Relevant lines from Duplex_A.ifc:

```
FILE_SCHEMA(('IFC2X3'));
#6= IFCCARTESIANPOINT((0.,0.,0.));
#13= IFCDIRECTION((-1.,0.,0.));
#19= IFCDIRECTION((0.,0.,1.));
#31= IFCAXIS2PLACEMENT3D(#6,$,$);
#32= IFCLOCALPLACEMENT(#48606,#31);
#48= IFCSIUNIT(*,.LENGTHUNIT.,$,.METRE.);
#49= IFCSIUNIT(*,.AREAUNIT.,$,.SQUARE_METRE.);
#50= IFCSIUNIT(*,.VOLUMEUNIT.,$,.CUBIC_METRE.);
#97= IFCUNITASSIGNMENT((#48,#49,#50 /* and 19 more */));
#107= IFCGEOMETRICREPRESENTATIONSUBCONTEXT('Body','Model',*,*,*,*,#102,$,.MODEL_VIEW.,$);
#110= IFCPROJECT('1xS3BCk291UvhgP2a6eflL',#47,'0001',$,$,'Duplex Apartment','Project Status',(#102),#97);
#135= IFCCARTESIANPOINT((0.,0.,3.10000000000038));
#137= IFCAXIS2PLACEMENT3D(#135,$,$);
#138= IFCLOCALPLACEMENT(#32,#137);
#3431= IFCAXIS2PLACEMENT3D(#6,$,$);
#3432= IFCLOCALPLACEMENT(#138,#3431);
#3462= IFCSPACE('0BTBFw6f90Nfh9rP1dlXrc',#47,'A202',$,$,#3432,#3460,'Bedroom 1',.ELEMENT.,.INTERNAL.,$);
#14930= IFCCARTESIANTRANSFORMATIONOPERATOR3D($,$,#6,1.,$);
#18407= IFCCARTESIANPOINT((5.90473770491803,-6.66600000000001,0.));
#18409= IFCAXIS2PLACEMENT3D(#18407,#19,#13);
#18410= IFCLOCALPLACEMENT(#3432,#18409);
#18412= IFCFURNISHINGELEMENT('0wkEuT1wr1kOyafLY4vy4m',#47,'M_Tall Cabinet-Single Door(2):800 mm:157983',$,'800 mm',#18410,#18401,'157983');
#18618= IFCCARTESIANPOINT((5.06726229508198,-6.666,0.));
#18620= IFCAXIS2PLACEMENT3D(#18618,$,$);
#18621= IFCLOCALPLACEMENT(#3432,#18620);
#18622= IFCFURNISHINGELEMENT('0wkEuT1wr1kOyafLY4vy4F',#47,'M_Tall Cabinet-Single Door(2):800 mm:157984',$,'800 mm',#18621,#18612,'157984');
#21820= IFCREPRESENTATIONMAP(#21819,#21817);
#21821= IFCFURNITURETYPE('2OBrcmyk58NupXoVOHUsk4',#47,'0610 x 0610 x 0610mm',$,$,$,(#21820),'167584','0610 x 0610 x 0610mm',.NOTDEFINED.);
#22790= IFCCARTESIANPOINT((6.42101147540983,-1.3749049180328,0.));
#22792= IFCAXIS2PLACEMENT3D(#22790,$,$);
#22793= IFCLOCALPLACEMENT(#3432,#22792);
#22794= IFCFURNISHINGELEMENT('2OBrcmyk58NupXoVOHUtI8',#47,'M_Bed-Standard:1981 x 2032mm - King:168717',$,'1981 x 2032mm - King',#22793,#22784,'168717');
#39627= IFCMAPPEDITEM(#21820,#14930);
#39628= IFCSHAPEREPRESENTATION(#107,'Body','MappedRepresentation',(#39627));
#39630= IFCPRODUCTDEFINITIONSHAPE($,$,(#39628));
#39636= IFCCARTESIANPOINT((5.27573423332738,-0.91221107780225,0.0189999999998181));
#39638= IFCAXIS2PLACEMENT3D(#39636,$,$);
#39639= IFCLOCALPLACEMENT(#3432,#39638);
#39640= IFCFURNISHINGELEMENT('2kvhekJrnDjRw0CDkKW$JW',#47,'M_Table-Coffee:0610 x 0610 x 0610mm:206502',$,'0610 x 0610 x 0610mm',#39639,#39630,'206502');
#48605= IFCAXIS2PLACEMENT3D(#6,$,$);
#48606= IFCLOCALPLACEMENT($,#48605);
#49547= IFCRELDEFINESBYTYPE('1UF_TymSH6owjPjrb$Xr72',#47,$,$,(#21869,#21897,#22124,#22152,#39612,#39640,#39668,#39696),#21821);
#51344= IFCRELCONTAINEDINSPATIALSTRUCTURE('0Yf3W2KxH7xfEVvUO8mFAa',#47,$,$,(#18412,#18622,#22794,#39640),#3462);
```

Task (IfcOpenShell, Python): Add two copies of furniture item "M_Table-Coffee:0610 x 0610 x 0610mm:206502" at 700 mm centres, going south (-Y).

```python
import numpy as np
import ifcopenshell
import ifcopenshell.api.geometry
import ifcopenshell.api.root
import ifcopenshell.util.element
import ifcopenshell.util.placement
import ifcopenshell.util.unit

model = ifcopenshell.open("Duplex_A.ifc")
unit_scale = ifcopenshell.util.unit.calculate_unit_scale(model)


def reuse_history(source, copy):
    """copy_class also copies each property set's owner history, people and application; keep the originals."""
    for rel in copy.IsDefinedBy:
        if rel.is_a("IfcRelDefinesByProperties") and (history := rel.RelatingPropertyDefinition.OwnerHistory):
            rel.RelatingPropertyDefinition.OwnerHistory = source.OwnerHistory
            ifcopenshell.util.element.remove_deep2(model, history)


source = model.by_id(39640)
base = ifcopenshell.util.placement.get_local_placement(source.ObjectPlacement)
step = np.array([0.0, -1.0, 0.0]) * 0.7 / unit_scale

for i in range(1, 3):
    copy = ifcopenshell.api.root.copy_class(model, product=source)
    copy.Representation = ifcopenshell.util.element.copy_deep(
        model, source.Representation, exclude=["IfcGeometricRepresentationContext", "IfcRepresentationMap"]
    )
    copy.Name = "M_Table-Coffee:0610 x 0610 x 0610mm"
    copy.Tag = None
    reuse_history(source, copy)
    matrix = base.copy()
    matrix[:3, 3] += i * step
    print("added at", matrix[:3, 3].round(3) + 0.0)
    ifcopenshell.api.geometry.edit_object_placement(model, product=copy, matrix=matrix, is_si=False)

model.write("Duplex_A_rev.ifc")
```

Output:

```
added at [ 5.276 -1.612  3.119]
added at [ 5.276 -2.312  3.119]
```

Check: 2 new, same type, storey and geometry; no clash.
